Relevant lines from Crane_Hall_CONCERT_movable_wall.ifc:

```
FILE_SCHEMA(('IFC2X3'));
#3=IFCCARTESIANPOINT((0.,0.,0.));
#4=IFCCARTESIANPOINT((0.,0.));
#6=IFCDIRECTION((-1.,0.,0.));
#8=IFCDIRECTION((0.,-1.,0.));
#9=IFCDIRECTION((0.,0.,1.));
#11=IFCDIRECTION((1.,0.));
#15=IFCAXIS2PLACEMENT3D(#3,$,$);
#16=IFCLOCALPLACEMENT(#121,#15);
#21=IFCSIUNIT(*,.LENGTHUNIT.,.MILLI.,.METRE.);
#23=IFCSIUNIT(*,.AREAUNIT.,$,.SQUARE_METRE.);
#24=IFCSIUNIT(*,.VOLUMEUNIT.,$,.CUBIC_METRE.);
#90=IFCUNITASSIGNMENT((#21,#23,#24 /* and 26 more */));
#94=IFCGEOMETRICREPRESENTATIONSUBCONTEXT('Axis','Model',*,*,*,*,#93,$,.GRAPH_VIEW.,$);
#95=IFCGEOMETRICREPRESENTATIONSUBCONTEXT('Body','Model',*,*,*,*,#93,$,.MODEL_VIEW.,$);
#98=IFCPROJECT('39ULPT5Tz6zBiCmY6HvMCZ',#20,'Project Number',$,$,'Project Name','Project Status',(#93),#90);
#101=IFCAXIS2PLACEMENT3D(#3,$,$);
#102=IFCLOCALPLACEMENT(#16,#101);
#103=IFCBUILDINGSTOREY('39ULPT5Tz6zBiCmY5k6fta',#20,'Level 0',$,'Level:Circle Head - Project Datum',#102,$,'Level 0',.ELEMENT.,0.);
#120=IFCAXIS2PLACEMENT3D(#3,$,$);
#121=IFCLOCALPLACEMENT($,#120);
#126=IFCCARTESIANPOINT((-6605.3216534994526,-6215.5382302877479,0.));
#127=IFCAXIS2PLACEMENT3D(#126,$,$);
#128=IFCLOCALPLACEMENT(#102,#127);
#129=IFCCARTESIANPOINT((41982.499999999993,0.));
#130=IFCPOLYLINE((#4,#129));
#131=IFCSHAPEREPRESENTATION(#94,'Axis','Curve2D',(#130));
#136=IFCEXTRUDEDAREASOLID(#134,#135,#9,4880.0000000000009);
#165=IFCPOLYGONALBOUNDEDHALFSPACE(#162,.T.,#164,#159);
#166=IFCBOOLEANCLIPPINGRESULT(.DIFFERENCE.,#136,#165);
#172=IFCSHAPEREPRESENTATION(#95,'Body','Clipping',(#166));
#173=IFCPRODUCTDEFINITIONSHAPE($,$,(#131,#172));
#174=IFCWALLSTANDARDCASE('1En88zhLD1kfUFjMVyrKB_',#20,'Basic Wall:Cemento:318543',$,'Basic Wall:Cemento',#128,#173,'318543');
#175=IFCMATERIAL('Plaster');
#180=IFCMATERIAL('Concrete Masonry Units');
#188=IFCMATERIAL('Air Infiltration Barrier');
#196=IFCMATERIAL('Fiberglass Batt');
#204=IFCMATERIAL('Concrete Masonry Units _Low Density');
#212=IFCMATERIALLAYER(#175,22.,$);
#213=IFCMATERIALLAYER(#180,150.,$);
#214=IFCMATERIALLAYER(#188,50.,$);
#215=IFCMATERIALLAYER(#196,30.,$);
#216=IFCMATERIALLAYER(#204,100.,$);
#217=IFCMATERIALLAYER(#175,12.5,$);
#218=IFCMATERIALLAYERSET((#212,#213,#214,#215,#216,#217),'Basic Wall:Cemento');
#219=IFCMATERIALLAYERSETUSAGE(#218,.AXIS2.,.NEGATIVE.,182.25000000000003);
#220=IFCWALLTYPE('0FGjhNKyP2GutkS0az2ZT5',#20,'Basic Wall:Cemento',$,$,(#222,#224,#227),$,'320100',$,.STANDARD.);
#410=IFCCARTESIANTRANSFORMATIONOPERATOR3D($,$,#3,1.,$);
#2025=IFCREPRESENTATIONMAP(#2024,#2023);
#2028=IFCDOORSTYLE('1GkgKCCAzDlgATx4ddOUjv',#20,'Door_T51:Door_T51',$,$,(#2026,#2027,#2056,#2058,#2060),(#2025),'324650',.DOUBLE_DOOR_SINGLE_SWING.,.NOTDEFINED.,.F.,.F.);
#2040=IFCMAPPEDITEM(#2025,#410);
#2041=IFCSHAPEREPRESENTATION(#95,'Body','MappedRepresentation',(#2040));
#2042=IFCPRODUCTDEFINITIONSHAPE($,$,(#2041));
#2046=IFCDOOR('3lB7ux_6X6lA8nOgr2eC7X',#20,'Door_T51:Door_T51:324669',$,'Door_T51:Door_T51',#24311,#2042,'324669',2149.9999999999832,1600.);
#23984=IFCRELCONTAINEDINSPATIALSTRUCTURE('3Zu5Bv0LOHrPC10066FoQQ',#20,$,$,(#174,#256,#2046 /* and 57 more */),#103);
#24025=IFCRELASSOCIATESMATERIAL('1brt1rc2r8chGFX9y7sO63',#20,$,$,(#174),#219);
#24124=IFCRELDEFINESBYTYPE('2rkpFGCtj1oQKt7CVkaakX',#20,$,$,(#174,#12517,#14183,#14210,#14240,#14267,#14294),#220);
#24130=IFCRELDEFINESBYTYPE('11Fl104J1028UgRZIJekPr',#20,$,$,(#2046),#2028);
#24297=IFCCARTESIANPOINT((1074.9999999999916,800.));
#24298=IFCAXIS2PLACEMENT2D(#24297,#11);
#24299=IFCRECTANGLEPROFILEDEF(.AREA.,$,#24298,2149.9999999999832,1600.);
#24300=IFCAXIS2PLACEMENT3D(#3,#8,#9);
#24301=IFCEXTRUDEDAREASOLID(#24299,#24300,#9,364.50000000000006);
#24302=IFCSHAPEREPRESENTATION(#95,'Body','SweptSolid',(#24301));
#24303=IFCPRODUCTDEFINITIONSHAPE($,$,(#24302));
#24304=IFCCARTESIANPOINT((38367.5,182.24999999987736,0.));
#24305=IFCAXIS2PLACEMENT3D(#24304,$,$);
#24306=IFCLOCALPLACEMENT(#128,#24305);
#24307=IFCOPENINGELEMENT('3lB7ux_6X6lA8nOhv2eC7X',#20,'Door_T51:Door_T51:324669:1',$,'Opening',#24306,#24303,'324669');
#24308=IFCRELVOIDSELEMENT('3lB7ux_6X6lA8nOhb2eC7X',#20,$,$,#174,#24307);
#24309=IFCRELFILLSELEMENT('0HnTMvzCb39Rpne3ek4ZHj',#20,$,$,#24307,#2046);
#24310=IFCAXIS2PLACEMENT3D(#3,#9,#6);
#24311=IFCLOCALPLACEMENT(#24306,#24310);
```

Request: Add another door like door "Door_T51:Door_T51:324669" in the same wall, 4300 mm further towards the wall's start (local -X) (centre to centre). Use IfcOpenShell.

```python
import ifcopenshell
import ifcopenshell.api.feature
import ifcopenshell.api.geometry
import ifcopenshell.api.root
import ifcopenshell.geom
import ifcopenshell.util.element
import ifcopenshell.util.placement
import ifcopenshell.util.shape
import ifcopenshell.util.unit

model = ifcopenshell.open("Crane_Hall_CONCERT_movable_wall.ifc")
unit_scale = ifcopenshell.util.unit.calculate_unit_scale(model)
settings = ifcopenshell.geom.settings()


def volume(element):
    """Net volume in cubic metres, openings subtracted."""
    shape = ifcopenshell.geom.create_shape(settings, element)
    return ifcopenshell.util.shape.get_volume(shape.geometry)


def reuse_history(source, copy):
    """copy_class also copies each property set's owner history, people and application; keep the originals."""
    for rel in copy.IsDefinedBy:
        if rel.is_a("IfcRelDefinesByProperties") and (history := rel.RelatingPropertyDefinition.OwnerHistory):
            rel.RelatingPropertyDefinition.OwnerHistory = source.OwnerHistory
            ifcopenshell.util.element.remove_deep2(model, history)


door = model.by_guid("3lB7ux_6X6lA8nOgr2eC7X")
opening = door.FillsVoids[0].RelatingOpeningElement
wall = opening.VoidsElements[0].RelatingBuildingElement
before = volume(wall)
shift = ifcopenshell.util.placement.get_local_placement(wall.ObjectPlacement)[:3, 0] * -4.3 / unit_scale

# copy_class copies the void relationship, type, container and properties, but no geometry.
new_opening = ifcopenshell.api.root.copy_class(model, product=opening)
new_opening.Representation = ifcopenshell.util.element.copy_deep(
    model, opening.Representation, exclude=["IfcGeometricRepresentationContext", "IfcRepresentationMap"]
)
new_opening.Name = "Door_T51:Door_T51"
new_opening.Tag = None
new_door = ifcopenshell.api.root.copy_class(model, product=door)
new_door.Representation = ifcopenshell.util.element.copy_deep(
    model, door.Representation, exclude=["IfcGeometricRepresentationContext", "IfcRepresentationMap"]
)
new_door.Name = "Door_T51:Door_T51"
new_door.Tag = None
reuse_history(door, new_door)
fills = ifcopenshell.api.feature.add_filling(model, opening=new_opening, element=new_door)
fills.OwnerHistory = new_door.OwnerHistory  # required in IFC2X3

for old, new in ((opening, new_opening), (door, new_door)):
    matrix = ifcopenshell.util.placement.get_local_placement(old.ObjectPlacement)
    matrix[:3, 3] += shift
    ifcopenshell.api.geometry.edit_object_placement(model, product=new, matrix=matrix, is_si=False)

after = volume(wall)

print(f"wall volume {before:.3f} -> {after:.3f} m3")

model.write("Crane_Hall_CONCERT_movable_wall_rev.ifc")
```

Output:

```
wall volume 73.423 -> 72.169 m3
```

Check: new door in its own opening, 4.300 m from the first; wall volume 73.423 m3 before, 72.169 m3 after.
